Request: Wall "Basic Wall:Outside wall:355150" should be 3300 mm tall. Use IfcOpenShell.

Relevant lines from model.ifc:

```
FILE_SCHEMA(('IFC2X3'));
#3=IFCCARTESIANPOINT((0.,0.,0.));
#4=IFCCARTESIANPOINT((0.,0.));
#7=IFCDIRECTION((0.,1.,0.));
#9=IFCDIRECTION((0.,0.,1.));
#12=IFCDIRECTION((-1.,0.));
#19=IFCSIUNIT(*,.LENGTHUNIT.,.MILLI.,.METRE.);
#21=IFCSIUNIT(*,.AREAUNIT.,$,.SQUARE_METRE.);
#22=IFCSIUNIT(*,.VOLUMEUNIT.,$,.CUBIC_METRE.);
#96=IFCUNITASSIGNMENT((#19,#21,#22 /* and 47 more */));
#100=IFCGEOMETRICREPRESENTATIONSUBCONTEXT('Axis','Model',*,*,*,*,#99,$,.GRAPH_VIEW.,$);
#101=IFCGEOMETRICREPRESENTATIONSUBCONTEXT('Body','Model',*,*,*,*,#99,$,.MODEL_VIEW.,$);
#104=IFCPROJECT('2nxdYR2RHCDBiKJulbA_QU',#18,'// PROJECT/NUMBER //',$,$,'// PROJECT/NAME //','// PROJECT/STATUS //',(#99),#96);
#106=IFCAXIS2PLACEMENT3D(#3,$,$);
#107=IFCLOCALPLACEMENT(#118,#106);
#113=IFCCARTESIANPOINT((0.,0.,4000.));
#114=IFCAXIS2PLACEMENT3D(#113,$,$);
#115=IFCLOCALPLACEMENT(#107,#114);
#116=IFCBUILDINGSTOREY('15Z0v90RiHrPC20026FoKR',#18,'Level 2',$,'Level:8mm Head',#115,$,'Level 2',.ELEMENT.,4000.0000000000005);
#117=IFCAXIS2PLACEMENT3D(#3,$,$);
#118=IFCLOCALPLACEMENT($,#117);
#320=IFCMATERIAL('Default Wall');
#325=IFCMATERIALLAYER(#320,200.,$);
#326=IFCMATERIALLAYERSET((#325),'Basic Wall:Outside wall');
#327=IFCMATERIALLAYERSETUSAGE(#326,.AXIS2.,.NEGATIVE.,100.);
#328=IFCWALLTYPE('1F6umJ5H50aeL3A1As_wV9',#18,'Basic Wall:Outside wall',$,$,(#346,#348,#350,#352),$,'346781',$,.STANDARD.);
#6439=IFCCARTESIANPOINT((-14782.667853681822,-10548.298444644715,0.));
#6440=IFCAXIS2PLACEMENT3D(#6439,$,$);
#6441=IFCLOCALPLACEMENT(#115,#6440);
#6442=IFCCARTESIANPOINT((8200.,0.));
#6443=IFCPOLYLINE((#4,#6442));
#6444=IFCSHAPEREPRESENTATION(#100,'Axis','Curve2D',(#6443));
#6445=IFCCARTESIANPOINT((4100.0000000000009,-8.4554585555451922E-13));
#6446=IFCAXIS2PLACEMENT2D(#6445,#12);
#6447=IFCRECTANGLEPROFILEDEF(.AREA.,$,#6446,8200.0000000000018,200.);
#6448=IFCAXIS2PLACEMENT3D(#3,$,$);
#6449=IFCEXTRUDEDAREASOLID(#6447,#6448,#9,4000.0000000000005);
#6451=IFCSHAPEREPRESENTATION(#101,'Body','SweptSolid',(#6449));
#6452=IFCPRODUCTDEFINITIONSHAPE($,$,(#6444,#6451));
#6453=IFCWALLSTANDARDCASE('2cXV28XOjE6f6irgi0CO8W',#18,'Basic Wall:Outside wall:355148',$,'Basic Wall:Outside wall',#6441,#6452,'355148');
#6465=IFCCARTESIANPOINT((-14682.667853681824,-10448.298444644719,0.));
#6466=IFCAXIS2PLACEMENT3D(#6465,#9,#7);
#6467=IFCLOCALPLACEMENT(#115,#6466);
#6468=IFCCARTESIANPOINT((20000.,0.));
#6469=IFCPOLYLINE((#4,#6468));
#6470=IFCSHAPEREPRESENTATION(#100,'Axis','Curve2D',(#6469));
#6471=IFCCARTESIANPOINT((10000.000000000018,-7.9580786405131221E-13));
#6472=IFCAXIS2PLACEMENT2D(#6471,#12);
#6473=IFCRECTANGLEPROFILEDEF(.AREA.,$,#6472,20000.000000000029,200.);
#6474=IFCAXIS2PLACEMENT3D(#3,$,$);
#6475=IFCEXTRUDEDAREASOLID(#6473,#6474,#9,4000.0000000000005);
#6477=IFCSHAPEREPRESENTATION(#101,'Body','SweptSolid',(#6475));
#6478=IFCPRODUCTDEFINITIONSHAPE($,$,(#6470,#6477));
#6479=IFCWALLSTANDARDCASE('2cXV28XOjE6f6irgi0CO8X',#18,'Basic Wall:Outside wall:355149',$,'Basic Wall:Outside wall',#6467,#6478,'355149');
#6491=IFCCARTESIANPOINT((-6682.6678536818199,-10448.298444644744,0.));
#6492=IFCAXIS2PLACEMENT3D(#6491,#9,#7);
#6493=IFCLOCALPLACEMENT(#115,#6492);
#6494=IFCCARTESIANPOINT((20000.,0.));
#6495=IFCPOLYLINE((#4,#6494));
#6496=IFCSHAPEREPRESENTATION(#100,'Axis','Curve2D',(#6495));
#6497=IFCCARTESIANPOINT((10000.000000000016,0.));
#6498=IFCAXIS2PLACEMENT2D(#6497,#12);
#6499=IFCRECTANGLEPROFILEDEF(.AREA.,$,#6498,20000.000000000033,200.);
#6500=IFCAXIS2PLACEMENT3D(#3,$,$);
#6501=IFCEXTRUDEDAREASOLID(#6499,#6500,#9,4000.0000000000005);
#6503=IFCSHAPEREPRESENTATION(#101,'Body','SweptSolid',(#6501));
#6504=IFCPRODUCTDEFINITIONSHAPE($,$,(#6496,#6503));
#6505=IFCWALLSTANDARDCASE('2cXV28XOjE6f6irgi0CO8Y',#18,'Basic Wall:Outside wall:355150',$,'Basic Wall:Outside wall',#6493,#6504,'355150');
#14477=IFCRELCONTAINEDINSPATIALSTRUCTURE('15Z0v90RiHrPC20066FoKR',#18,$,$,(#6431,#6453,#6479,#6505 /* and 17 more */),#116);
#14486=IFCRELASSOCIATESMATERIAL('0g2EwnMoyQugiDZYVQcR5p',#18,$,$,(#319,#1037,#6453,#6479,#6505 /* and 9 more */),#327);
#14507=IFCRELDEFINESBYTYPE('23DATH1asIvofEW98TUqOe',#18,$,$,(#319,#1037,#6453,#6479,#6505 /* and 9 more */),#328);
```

```python
import ifcopenshell
import ifcopenshell.geom
import ifcopenshell.util.representation
import ifcopenshell.util.shape
import ifcopenshell.util.unit

model = ifcopenshell.open("model.ifc")
unit_scale = ifcopenshell.util.unit.calculate_unit_scale(model)
settings = ifcopenshell.geom.settings()


def volume(element):
    """Net volume in cubic metres, openings subtracted."""
    shape = ifcopenshell.geom.create_shape(settings, element)
    return ifcopenshell.util.shape.get_volume(shape.geometry)


wall = model.by_guid("2cXV28XOjE6f6irgi0CO8Y")
before = volume(wall)

body = ifcopenshell.util.representation.get_representation(wall, "Model", "Body")
solid = body.Items[0]
old_height = solid.Depth
solid.Depth = 3.3 / unit_scale
after = volume(wall)

print(f"height {old_height:g} -> {solid.Depth:g}, volume {before:.3f} -> {after:.3f} m3")

model.write("model_edited.ifc")
```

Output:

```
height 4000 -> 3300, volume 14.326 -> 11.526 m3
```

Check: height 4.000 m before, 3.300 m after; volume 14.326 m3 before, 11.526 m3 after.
